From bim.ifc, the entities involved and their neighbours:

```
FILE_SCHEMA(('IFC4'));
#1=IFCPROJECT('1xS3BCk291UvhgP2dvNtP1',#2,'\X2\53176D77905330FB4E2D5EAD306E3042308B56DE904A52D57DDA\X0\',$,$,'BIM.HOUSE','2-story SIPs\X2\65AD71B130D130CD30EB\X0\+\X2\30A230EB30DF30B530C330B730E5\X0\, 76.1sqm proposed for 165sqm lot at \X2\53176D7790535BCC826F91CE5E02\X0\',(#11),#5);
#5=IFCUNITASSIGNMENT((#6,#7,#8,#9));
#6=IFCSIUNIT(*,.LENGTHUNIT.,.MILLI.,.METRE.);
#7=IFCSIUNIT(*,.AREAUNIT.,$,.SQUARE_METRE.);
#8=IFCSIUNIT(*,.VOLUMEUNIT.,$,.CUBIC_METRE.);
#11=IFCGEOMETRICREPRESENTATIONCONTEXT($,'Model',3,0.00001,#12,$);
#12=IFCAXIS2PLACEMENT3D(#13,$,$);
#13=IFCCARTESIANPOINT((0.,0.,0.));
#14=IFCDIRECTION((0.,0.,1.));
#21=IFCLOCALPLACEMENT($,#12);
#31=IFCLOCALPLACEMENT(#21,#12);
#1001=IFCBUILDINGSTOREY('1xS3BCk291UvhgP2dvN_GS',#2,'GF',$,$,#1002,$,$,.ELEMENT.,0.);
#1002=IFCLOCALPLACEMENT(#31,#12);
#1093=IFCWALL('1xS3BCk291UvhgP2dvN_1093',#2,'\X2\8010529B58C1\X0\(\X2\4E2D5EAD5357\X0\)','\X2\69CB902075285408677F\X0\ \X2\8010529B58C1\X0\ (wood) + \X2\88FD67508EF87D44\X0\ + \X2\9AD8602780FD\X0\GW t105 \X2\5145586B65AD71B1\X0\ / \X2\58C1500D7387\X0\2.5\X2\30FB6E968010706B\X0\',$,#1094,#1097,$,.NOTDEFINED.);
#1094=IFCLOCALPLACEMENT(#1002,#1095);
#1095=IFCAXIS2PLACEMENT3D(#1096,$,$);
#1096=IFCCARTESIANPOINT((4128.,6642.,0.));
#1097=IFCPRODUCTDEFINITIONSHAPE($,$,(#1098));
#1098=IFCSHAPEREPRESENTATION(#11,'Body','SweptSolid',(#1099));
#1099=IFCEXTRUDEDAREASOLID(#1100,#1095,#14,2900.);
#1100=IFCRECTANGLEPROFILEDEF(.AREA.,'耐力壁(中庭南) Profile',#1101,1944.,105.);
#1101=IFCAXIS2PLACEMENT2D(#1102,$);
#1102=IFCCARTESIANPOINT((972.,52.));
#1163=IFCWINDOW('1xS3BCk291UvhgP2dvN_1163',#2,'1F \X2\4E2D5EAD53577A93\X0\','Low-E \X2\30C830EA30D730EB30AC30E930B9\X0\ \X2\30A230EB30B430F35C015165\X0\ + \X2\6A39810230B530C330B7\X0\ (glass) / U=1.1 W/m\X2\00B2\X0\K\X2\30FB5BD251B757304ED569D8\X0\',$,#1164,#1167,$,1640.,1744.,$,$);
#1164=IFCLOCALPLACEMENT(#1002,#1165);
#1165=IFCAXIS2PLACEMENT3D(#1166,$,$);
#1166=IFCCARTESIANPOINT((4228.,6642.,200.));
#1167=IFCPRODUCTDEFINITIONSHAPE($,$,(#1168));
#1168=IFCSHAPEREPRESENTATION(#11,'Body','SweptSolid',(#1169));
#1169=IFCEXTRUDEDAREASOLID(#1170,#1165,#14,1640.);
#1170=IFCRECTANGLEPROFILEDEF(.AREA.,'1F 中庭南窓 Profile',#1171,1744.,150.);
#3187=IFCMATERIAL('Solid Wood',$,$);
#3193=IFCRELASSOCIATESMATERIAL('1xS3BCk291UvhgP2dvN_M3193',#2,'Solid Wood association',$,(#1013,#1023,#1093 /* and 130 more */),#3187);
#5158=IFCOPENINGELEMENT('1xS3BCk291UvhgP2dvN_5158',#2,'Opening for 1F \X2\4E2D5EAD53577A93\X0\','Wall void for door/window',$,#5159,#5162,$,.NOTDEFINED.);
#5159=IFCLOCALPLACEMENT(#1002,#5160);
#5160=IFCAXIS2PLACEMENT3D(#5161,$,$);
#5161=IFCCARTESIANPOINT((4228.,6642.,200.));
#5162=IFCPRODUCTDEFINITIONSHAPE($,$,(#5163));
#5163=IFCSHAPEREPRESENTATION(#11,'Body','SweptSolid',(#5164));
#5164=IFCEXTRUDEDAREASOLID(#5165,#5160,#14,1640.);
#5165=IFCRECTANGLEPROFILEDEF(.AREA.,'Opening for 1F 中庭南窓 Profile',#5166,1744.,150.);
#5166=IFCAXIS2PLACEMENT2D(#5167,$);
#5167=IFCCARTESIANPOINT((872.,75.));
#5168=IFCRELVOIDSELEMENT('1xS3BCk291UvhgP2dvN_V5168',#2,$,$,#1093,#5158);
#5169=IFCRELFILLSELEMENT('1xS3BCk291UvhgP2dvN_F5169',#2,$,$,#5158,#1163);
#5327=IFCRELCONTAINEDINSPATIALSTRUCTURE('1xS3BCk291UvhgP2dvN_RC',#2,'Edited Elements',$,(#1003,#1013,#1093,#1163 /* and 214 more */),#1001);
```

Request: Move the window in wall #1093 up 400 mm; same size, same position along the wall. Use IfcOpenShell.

```python
import numpy as np
import ifcopenshell
import ifcopenshell.api.geometry
import ifcopenshell.util.placement
import ifcopenshell.util.unit

model = ifcopenshell.open("bim.ifc")
unit_scale = ifcopenshell.util.unit.calculate_unit_scale(model)

window = model.by_guid("1xS3BCk291UvhgP2dvN_1163")
opening = window.FillsVoids[0].RelatingOpeningElement
dz = 400.0

shift = np.array([0.0, 0.0, dz])
# The window is not placed relative to its opening, so move both.
for product in (opening, window):
    matrix = ifcopenshell.util.placement.get_local_placement(product.ObjectPlacement)
    matrix[:3, 3] += shift
    ifcopenshell.api.geometry.edit_object_placement(model, product=product, matrix=matrix, is_si=False)

print(f"moved by {dz * unit_scale:+.3f} m")

model.write("bim_updated.ifc")
```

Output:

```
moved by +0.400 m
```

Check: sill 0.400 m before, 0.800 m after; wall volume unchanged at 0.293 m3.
